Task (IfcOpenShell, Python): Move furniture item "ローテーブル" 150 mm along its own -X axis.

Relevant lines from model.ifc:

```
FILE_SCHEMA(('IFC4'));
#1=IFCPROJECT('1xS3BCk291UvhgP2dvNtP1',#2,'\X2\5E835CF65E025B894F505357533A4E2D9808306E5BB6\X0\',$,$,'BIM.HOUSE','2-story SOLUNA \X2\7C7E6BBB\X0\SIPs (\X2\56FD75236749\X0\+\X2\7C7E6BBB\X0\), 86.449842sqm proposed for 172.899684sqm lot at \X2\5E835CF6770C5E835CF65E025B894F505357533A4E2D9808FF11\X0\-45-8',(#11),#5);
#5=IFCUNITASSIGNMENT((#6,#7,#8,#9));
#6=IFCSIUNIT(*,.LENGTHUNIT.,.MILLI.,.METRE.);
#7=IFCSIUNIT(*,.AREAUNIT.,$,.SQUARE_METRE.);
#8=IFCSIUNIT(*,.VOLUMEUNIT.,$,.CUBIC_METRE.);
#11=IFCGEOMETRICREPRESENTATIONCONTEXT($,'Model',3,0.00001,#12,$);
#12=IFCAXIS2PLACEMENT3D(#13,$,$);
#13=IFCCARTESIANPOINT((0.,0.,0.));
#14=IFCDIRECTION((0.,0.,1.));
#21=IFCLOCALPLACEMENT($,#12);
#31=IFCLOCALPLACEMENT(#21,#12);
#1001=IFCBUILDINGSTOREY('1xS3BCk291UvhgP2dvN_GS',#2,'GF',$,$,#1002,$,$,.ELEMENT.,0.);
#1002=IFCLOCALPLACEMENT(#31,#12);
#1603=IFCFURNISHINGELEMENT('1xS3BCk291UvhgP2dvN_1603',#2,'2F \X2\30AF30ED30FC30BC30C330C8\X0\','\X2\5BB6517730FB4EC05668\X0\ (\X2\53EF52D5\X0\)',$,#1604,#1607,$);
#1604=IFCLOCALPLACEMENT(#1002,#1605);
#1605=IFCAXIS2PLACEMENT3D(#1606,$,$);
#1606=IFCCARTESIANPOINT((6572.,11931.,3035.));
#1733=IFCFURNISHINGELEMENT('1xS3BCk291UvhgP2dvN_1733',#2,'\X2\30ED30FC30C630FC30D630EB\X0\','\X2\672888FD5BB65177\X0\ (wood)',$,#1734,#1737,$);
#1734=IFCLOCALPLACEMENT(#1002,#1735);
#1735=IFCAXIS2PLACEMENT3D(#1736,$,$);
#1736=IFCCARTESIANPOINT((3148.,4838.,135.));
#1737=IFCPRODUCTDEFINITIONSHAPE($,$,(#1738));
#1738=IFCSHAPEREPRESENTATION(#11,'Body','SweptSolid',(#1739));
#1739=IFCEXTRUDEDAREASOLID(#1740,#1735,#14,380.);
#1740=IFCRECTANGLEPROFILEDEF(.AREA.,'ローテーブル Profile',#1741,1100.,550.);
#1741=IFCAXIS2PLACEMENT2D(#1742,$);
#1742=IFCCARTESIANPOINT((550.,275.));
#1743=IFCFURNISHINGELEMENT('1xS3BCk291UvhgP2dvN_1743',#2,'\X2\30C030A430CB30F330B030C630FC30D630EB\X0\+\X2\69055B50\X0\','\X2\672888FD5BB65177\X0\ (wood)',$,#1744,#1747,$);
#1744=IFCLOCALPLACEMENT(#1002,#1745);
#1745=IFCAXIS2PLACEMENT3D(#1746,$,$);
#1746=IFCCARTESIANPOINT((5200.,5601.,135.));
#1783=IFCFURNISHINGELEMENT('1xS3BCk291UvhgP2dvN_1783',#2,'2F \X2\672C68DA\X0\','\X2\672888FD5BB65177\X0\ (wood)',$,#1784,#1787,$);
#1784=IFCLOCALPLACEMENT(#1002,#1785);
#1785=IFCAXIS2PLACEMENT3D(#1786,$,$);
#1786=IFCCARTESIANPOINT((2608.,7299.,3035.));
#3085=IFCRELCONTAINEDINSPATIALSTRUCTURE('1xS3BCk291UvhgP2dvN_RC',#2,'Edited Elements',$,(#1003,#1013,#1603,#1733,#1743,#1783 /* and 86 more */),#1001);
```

```python
import ifcopenshell
import ifcopenshell.api.geometry
import ifcopenshell.util.placement

model = ifcopenshell.open("model.ifc")

item = model.by_guid("1xS3BCk291UvhgP2dvN_1733")
matrix = ifcopenshell.util.placement.get_local_placement(item.ObjectPlacement)
matrix[:3, 3] -= matrix[:3, 0] * 150.0
ifcopenshell.api.geometry.edit_object_placement(model, product=item, matrix=matrix, is_si=False)

print(ifcopenshell.util.placement.get_local_placement(item.ObjectPlacement).round(3) + 0.0)

model.write("model_rev.ifc")
```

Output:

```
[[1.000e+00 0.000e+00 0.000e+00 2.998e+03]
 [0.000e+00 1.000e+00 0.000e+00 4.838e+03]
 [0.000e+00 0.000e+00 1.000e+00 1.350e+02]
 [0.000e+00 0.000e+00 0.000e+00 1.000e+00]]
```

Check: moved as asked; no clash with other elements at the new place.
